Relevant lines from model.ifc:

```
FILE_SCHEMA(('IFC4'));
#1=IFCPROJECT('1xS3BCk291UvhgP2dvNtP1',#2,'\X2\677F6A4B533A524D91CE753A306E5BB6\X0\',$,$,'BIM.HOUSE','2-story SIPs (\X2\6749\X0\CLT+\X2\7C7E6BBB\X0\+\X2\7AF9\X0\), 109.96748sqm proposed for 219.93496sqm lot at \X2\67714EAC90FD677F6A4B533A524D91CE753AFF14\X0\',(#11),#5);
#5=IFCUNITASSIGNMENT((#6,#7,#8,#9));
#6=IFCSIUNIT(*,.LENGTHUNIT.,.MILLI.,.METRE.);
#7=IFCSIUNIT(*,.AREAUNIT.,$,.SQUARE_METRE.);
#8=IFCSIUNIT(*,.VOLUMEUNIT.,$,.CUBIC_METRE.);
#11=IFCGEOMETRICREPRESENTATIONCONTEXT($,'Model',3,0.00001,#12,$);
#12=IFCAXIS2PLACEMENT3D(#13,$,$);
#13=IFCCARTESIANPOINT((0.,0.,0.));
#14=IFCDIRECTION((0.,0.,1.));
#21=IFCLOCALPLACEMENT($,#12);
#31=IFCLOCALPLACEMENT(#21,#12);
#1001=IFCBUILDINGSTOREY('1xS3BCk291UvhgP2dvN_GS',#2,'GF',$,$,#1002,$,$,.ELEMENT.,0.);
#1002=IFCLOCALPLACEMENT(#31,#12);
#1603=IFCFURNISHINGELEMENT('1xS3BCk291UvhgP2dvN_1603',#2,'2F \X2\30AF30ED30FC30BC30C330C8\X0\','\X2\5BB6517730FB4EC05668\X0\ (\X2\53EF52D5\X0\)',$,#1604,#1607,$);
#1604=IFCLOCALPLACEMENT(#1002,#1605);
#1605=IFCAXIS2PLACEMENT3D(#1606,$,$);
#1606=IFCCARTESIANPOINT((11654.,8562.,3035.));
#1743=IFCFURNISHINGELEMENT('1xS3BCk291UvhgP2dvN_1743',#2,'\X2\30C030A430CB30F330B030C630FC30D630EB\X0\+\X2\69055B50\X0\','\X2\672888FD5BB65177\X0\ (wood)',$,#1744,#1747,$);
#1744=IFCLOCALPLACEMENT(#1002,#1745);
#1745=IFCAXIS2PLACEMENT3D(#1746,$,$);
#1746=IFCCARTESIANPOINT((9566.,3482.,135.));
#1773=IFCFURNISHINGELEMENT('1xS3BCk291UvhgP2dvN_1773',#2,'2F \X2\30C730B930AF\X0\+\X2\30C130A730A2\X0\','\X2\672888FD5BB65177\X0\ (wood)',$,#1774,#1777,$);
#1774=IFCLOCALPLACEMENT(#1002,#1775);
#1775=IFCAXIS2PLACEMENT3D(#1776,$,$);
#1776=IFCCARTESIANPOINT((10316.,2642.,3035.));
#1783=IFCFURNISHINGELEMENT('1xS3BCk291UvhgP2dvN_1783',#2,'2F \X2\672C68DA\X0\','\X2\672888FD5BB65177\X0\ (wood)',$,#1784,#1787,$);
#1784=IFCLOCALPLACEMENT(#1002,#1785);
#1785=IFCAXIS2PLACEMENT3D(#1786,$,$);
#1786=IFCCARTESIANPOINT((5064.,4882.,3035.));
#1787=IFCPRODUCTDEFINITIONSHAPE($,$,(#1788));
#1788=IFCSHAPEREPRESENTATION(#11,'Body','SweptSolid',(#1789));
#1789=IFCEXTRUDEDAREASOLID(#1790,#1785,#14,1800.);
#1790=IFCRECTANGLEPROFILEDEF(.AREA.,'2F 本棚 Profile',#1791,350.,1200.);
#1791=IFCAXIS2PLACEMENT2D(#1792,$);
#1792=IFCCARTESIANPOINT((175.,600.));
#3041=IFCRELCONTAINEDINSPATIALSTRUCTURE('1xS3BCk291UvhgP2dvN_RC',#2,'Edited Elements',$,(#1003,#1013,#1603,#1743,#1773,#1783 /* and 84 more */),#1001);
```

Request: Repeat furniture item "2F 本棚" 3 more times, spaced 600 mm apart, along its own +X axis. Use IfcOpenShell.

```python
import ifcopenshell
import ifcopenshell.api.geometry
import ifcopenshell.api.root
import ifcopenshell.util.element
import ifcopenshell.util.placement
import ifcopenshell.util.unit

model = ifcopenshell.open("model.ifc")
unit_scale = ifcopenshell.util.unit.calculate_unit_scale(model)


def reuse_history(source, copy):
    """copy_class also copies each property set's owner history, people and application; keep the originals."""
    for rel in copy.IsDefinedBy:
        if rel.is_a("IfcRelDefinesByProperties") and (history := rel.RelatingPropertyDefinition.OwnerHistory):
            rel.RelatingPropertyDefinition.OwnerHistory = source.OwnerHistory
            ifcopenshell.util.element.remove_deep2(model, history)


source = model.by_id(1783)
base = ifcopenshell.util.placement.get_local_placement(source.ObjectPlacement)
step = base[:3, 0] * 0.6 / unit_scale

for i in range(1, 4):
    copy = ifcopenshell.api.root.copy_class(model, product=source)
    copy.Representation = ifcopenshell.util.element.copy_deep(
        model, source.Representation, exclude=["IfcGeometricRepresentationContext", "IfcRepresentationMap"]
    )
    reuse_history(source, copy)
    matrix = base.copy()
    matrix[:3, 3] += i * step
    print("added at", matrix[:3, 3].round(3) + 0.0)
    ifcopenshell.api.geometry.edit_object_placement(model, product=copy, matrix=matrix, is_si=False)

model.write("model-out.ifc")
```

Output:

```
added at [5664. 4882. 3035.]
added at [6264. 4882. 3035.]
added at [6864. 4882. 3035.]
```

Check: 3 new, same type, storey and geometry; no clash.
